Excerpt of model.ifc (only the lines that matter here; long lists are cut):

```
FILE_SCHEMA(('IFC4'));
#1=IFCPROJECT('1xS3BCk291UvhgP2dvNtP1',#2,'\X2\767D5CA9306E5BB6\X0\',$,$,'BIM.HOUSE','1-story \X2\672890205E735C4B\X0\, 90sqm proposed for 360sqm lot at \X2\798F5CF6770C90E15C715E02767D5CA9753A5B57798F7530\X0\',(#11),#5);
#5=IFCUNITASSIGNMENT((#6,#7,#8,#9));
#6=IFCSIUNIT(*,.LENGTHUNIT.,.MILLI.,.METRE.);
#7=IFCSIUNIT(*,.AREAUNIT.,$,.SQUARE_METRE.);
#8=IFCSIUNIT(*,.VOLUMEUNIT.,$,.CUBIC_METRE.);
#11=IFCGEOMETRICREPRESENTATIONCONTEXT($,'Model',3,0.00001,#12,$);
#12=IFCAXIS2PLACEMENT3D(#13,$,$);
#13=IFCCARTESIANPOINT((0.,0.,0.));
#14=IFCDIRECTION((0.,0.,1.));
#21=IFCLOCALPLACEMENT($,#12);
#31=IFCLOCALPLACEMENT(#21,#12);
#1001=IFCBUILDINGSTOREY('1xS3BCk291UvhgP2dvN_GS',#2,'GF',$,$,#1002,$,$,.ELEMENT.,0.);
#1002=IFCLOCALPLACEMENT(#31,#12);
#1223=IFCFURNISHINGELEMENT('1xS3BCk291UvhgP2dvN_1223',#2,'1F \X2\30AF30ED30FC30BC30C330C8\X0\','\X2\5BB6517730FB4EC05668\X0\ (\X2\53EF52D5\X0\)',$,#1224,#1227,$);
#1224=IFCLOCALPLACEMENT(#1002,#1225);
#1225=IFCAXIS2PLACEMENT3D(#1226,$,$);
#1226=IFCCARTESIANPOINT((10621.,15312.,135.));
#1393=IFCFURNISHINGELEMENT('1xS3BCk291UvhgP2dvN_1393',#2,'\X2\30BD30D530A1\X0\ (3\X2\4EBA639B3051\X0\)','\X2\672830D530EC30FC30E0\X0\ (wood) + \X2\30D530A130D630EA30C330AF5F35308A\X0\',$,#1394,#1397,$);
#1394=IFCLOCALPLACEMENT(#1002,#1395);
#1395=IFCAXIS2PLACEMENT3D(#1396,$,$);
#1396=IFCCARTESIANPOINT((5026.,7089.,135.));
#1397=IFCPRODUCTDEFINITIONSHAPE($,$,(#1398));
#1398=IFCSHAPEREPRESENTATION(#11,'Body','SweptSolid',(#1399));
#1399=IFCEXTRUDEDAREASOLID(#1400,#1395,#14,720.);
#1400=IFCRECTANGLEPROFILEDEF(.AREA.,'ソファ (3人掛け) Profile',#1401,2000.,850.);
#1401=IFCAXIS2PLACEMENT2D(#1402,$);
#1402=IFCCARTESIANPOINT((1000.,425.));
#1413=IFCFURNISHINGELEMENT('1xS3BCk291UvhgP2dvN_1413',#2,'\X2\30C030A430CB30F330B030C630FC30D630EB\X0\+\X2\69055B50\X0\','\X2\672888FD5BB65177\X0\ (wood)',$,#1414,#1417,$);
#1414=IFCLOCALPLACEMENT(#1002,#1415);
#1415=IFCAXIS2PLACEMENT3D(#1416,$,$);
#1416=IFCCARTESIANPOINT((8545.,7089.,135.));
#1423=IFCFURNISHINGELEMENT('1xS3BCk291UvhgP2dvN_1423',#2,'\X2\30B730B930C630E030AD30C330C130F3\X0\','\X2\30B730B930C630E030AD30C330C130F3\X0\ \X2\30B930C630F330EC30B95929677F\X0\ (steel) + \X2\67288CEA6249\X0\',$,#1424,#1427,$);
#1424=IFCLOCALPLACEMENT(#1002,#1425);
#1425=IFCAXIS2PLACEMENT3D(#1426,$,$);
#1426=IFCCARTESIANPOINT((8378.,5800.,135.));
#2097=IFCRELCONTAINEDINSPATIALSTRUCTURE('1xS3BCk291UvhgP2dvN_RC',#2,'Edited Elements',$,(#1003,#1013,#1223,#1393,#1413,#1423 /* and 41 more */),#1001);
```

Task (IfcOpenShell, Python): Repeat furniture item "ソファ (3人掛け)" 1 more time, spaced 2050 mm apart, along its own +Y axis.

```python
import ifcopenshell
import ifcopenshell.api.geometry
import ifcopenshell.api.root
import ifcopenshell.util.element
import ifcopenshell.util.placement

model = ifcopenshell.open("model.ifc")


def reuse_history(source, copy):
    """copy_class also copies each property set's owner history, people and application; keep the originals."""
    for rel in copy.IsDefinedBy:
        if rel.is_a("IfcRelDefinesByProperties") and (history := rel.RelatingPropertyDefinition.OwnerHistory):
            rel.RelatingPropertyDefinition.OwnerHistory = source.OwnerHistory
            ifcopenshell.util.element.remove_deep2(model, history)


source = model.by_guid("1xS3BCk291UvhgP2dvN_1393")
base = ifcopenshell.util.placement.get_local_placement(source.ObjectPlacement)
step = base[:3, 1] * 2050.0

for i in range(1, 2):
    copy = ifcopenshell.api.root.copy_class(model, product=source)
    copy.Representation = ifcopenshell.util.element.copy_deep(
        model, source.Representation, exclude=["IfcGeometricRepresentationContext", "IfcRepresentationMap"]
    )
    reuse_history(source, copy)
    matrix = base.copy()
    matrix[:3, 3] += i * step
    print("added at", matrix[:3, 3].round(3) + 0.0)
    ifcopenshell.api.geometry.edit_object_placement(model, product=copy, matrix=matrix, is_si=False)

model.write("model_edited.ifc")
```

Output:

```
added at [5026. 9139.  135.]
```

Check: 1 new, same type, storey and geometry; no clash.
